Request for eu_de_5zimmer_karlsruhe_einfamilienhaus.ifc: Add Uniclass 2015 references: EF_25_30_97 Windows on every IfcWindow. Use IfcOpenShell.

First a look at what the model holds.

```python
import ifcopenshell

model = ifcopenshell.open("eu_de_5zimmer_karlsruhe_einfamilienhaus.ifc")
print(model.schema)
print("classifications:", [c.Name for c in model.by_type("IfcClassification")])
for ifc_class in ("IfcDoor", "IfcRoof", "IfcStair", "IfcWall", "IfcWindow"):
    print(ifc_class, len(model.by_type(ifc_class)))
```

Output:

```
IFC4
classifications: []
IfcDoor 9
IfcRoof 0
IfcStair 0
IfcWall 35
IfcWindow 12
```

```python
import ifcopenshell
import ifcopenshell.api.classification

model = ifcopenshell.open("eu_de_5zimmer_karlsruhe_einfamilienhaus.ifc")

system = ifcopenshell.api.classification.add_classification(model, classification="Uniclass 2015")

codes = {
    "IfcWindow": ("EF_25_30_97", "Windows"),
}
for ifc_class, (code, name) in codes.items():
    products = model.by_type(ifc_class)
    ifcopenshell.api.classification.add_reference(
        model, products=products, classification=system, identification=code, name=name
    )
    print(code, len(products))

model.write("eu_de_5zimmer_karlsruhe_einfamilienhaus_rev.ifc")
```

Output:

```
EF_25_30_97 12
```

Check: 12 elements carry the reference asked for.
